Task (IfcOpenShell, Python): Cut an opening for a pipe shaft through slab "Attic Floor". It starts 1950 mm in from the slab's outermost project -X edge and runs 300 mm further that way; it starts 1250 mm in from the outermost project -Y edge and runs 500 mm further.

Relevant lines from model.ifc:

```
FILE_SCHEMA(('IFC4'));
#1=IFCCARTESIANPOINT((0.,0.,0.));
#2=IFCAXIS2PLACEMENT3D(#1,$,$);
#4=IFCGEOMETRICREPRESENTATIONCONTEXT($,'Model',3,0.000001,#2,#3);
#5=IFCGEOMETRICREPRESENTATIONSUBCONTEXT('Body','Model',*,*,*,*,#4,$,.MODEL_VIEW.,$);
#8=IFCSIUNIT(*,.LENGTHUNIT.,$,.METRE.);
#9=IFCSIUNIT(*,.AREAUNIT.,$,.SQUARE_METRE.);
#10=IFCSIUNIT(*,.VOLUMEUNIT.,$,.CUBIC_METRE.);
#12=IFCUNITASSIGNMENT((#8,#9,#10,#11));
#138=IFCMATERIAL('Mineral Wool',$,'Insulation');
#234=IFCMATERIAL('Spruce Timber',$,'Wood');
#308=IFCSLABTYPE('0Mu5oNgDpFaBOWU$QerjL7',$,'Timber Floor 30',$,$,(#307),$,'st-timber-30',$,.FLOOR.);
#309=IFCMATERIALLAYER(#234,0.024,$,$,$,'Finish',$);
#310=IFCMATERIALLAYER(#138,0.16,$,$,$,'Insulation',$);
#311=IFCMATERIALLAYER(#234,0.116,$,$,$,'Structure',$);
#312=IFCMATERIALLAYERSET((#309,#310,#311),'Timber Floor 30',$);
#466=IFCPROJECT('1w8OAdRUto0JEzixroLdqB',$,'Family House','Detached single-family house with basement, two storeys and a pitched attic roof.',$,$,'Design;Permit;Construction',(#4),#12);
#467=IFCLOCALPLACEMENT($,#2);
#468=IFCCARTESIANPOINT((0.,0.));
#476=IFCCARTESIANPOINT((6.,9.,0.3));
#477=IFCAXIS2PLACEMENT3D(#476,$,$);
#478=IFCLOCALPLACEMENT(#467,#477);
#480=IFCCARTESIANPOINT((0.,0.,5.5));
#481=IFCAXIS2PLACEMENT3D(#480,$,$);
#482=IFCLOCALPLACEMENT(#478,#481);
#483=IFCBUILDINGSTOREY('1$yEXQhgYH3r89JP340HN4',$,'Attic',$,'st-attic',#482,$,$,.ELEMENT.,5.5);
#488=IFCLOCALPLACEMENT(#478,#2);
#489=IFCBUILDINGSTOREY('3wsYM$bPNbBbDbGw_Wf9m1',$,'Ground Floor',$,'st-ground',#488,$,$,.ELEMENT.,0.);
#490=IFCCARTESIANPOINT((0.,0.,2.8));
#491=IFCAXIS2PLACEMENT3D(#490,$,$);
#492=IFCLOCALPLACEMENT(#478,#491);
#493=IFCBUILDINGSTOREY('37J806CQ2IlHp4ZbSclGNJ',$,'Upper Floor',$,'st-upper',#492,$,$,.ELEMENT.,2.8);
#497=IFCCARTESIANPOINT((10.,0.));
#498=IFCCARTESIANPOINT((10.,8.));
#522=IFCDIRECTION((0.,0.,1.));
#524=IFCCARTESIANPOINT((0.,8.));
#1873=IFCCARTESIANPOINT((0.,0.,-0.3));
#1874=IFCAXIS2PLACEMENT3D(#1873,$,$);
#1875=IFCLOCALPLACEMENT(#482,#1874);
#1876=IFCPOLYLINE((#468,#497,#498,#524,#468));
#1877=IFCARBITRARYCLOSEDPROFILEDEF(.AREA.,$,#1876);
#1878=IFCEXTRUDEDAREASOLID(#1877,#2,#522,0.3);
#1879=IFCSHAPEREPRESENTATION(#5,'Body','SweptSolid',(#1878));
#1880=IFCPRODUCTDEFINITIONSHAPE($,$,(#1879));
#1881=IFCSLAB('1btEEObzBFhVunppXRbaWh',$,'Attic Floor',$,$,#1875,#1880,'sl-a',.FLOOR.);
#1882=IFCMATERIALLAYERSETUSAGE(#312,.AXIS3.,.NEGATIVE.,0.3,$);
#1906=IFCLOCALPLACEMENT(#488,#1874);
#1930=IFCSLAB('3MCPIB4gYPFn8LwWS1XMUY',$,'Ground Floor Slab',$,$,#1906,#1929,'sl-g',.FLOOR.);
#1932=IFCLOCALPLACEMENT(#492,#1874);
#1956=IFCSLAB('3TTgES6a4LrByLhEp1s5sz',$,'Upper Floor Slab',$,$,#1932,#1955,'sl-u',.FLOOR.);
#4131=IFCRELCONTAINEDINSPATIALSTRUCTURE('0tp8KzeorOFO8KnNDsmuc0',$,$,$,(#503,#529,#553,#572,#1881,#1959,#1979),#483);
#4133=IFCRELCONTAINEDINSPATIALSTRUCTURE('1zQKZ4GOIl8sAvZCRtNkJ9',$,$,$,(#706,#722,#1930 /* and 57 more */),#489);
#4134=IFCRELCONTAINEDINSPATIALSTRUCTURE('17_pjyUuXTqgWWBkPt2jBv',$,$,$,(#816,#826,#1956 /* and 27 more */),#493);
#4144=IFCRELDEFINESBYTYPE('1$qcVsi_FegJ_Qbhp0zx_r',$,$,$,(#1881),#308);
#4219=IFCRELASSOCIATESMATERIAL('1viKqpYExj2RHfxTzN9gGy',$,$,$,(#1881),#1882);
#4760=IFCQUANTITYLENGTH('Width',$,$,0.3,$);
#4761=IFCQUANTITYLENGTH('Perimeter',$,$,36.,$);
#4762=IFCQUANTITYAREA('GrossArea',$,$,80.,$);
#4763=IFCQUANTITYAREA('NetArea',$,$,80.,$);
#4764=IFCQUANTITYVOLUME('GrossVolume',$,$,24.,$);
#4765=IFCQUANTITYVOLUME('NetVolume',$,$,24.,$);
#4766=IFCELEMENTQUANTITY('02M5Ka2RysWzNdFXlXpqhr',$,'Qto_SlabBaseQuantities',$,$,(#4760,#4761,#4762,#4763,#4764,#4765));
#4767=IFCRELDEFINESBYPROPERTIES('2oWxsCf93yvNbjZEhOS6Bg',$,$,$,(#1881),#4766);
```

```python
import numpy as np
import ifcopenshell
import ifcopenshell.api.feature
import ifcopenshell.api.geometry
import ifcopenshell.api.pset
import ifcopenshell.api.root
import ifcopenshell.geom
import ifcopenshell.util.element
import ifcopenshell.util.placement
import ifcopenshell.util.representation
import ifcopenshell.util.shape
import ifcopenshell.util.unit

model = ifcopenshell.open("model.ifc")
unit_scale = ifcopenshell.util.unit.calculate_unit_scale(model)
area_scale = ifcopenshell.util.unit.calculate_unit_scale(model, "AREAUNIT")
volume_scale = ifcopenshell.util.unit.calculate_unit_scale(model, "VOLUMEUNIT")
settings = ifcopenshell.geom.settings()


def volume(element):
    """Net volume in cubic metres, openings subtracted."""
    shape = ifcopenshell.geom.create_shape(settings, element)
    return ifcopenshell.util.shape.get_volume(shape.geometry)


slab = model.by_id(1881)
before = volume(slab)

# Extent in the slab's own axes, in metres. The edges named are its -X and -Y sides.
slab_shape = ifcopenshell.geom.create_shape(settings, slab)
vertices = ifcopenshell.util.shape.get_vertices(slab_shape.geometry)
x_min, y_min, bottom = vertices.min(axis=0)
top = vertices[:, 2].max()

opening = ifcopenshell.api.root.create_entity(model, ifc_class="IfcOpeningElement", name="Pipe shaft opening", predefined_type="OPENING")
context = ifcopenshell.util.representation.get_context(model, "Model", "Body", "MODEL_VIEW")
width, depth = 0.3, 0.5
outline = [(0.0, 0.0), (width, 0.0), (width, depth), (0.0, depth), (0.0, 0.0)]
# Overshoot both faces by 50 mm so the cut is clean.
shape = ifcopenshell.api.geometry.add_slab_representation(
    model, context=context, depth=top - bottom + 0.1, polyline=outline
)
ifcopenshell.api.geometry.assign_representation(model, product=opening, representation=shape)

matrix = ifcopenshell.util.placement.get_local_placement(slab.ObjectPlacement)
matrix[:, 3] = matrix @ np.append(np.array([x_min + 1.95, y_min + 1.25, bottom - 0.05]) / unit_scale, 1.0)
ifcopenshell.api.geometry.edit_object_placement(model, product=opening, matrix=matrix, is_si=False)
ifcopenshell.api.feature.add_feature(model, feature=opening, element=slab)

after = volume(slab)

# Update the slab's stored quantities.
qto = model.by_id(ifcopenshell.util.element.get_pset(slab, "Qto_SlabBaseQuantities", should_inherit=False)["id"])
ifcopenshell.api.pset.edit_qto(model, qto=qto, properties={
    "NetArea": after / (top - bottom) / area_scale,
    "NetVolume": after / volume_scale,
})

print(f"slab volume {before:.3f} -> {after:.3f} m3")

model.write("model_v2.ifc")
```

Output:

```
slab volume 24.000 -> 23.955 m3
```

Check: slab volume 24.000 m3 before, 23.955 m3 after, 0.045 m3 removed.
